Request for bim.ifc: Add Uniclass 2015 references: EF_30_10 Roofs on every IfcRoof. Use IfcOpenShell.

First a look at what the model holds.

```python
import ifcopenshell

model = ifcopenshell.open("bim.ifc")
print(model.schema)
print("classifications:", [c.Name for c in model.by_type("IfcClassification")])
for ifc_class in ("IfcDoor", "IfcRoof", "IfcStair", "IfcWall", "IfcWindow"):
    print(ifc_class, len(model.by_type(ifc_class)))
```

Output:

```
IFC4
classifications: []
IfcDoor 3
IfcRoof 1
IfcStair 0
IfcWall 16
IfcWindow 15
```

```python
import ifcopenshell
import ifcopenshell.api.classification

model = ifcopenshell.open("bim.ifc")

system = ifcopenshell.api.classification.add_classification(model, classification="Uniclass 2015")

codes = {
    "IfcRoof": ("EF_30_10", "Roofs"),
}
for ifc_class, (code, name) in codes.items():
    products = model.by_type(ifc_class)
    ifcopenshell.api.classification.add_reference(
        model, products=products, classification=system, identification=code, name=name
    )
    print(code, len(products))

model.write("bim_edited.ifc")
```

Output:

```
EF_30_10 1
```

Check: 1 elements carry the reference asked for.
